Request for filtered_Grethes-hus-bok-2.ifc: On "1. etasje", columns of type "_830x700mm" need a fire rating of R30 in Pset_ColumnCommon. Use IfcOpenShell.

First a look at what the model holds.

```python
import ifcopenshell
import ifcopenshell.util.element

model = ifcopenshell.open("filtered_Grethes-hus-bok-2.ifc")
print(model.schema)
storey = next(s for s in model.by_type("IfcBuildingStorey") if s.Name == "1. etasje")
columns = [e for e in ifcopenshell.util.element.get_decomposition(storey) if e.is_a("IfcColumn")]
seen = {}
for e in columns:
    element_type = ifcopenshell.util.element.get_type(e)
    key = (element_type.Name if element_type != e and element_type else None, ifcopenshell.util.element.get_pset(e, "Pset_ColumnCommon", "FireRating"))
    seen[key] = seen.get(key, 0) + 1
for (name, value), count in sorted(seen.items(), key=str):
    print(count, "x", name, "|", value)
```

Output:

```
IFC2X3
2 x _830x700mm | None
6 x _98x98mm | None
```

```python
import ifcopenshell
import ifcopenshell.api.pset
import ifcopenshell.util.element

model = ifcopenshell.open("filtered_Grethes-hus-bok-2.ifc")

storey = next(s for s in model.by_type("IfcBuildingStorey") if s.Name == "1. etasje")
columns = [e for e in ifcopenshell.util.element.get_decomposition(storey) if e.is_a("IfcColumn")]

count = 0
for e in columns:
    element_type = ifcopenshell.util.element.get_type(e)
    if element_type in (None, e) or element_type.Name != "_830x700mm":
        continue
    # add_pset returns the element's existing set when there is one.
    pset = ifcopenshell.api.pset.add_pset(model, product=e, name="Pset_ColumnCommon")
    ifcopenshell.api.pset.edit_pset(model, pset=pset, properties={"FireRating": "R30"})
    count += 1

print(count, "columns updated")

model.write("filtered_Grethes-hus-bok-2_rev.ifc")
```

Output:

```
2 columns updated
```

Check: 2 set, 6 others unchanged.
